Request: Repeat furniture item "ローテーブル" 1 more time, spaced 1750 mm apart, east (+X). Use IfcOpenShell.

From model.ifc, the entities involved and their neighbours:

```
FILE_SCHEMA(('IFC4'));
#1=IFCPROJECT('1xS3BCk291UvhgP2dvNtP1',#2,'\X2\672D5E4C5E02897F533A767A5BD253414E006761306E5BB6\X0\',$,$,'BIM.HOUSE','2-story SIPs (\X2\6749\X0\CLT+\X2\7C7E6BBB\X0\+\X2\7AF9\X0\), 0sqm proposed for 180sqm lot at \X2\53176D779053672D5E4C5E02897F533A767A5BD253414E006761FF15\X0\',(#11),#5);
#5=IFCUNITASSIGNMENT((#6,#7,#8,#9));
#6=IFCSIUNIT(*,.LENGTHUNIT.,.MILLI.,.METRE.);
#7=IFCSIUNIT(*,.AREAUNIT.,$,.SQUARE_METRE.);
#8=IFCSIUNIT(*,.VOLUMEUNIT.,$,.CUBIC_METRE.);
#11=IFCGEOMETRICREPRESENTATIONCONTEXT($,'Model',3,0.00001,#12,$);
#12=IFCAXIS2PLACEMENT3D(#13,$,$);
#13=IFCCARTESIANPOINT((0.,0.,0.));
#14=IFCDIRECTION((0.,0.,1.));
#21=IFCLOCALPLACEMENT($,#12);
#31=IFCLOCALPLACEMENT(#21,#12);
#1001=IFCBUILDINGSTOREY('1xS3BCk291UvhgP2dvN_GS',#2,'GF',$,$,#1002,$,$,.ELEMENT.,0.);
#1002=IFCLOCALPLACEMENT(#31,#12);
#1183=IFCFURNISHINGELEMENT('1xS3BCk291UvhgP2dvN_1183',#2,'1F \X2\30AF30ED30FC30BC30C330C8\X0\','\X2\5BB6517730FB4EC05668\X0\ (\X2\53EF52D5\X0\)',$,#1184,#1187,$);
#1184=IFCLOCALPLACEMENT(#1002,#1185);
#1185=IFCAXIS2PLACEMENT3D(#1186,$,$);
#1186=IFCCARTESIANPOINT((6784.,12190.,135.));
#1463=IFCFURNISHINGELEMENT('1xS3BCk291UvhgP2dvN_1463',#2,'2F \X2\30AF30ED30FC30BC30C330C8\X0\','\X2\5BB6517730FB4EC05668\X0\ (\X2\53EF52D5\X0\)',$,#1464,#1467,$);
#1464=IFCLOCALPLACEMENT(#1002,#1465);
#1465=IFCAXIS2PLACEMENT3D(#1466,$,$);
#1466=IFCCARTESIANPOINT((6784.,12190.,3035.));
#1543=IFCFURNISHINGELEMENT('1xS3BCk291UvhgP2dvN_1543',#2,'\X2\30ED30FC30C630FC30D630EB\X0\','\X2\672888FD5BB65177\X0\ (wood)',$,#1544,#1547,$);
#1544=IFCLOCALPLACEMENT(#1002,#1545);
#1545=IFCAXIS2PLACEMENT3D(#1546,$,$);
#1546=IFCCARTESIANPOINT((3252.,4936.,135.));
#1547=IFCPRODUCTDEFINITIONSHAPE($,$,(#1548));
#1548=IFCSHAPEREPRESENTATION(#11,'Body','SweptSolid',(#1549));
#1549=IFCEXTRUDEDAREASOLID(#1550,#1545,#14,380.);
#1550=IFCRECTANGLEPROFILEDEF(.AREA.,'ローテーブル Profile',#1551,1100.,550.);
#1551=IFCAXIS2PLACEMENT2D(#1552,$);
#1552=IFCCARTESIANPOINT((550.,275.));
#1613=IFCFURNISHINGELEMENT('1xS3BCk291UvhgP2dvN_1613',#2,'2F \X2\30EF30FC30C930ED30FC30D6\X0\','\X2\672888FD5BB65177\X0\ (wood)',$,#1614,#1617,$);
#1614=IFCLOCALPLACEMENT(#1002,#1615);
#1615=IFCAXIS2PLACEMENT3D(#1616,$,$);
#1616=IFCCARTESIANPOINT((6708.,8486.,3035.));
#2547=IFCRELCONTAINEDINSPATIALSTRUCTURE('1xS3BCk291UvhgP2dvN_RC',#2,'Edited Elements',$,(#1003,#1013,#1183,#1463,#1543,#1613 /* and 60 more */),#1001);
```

```python
import numpy as np
import ifcopenshell
import ifcopenshell.api.geometry
import ifcopenshell.api.root
import ifcopenshell.util.element
import ifcopenshell.util.placement
import ifcopenshell.util.unit

model = ifcopenshell.open("model.ifc")
unit_scale = ifcopenshell.util.unit.calculate_unit_scale(model)


def reuse_history(source, copy):
    """copy_class also copies each property set's owner history, people and application; keep the originals."""
    for rel in copy.IsDefinedBy:
        if rel.is_a("IfcRelDefinesByProperties") and (history := rel.RelatingPropertyDefinition.OwnerHistory):
            rel.RelatingPropertyDefinition.OwnerHistory = source.OwnerHistory
            ifcopenshell.util.element.remove_deep2(model, history)


source = model.by_guid("1xS3BCk291UvhgP2dvN_1543")
base = ifcopenshell.util.placement.get_local_placement(source.ObjectPlacement)
step = np.array([1.0, 0.0, 0.0]) * 1.75 / unit_scale

for i in range(1, 2):
    copy = ifcopenshell.api.root.copy_class(model, product=source)
    copy.Representation = ifcopenshell.util.element.copy_deep(
        model, source.Representation, exclude=["IfcGeometricRepresentationContext", "IfcRepresentationMap"]
    )
    reuse_history(source, copy)
    matrix = base.copy()
    matrix[:3, 3] += i * step
    print("added at", matrix[:3, 3].round(3) + 0.0)
    ifcopenshell.api.geometry.edit_object_placement(model, product=copy, matrix=matrix, is_si=False)

model.write("model_updated.ifc")
```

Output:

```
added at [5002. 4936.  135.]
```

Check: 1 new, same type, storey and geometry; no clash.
